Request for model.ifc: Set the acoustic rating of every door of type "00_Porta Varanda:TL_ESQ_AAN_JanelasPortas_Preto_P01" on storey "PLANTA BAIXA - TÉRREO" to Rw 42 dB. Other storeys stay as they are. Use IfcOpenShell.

First a look at what the model holds.

```python
import ifcopenshell
import ifcopenshell.util.element

model = ifcopenshell.open("model.ifc")
print(model.schema)
storey = next(s for s in model.by_type("IfcBuildingStorey") if s.Name == "PLANTA BAIXA - TÉRREO")
doors = [e for e in ifcopenshell.util.element.get_decomposition(storey) if e.is_a("IfcDoor")]
seen = {}
for e in doors:
    element_type = ifcopenshell.util.element.get_type(e)
    key = (element_type.Name if element_type != e and element_type else None, ifcopenshell.util.element.get_pset(e, "Pset_DoorCommon", "AcousticRating"))
    seen[key] = seen.get(key, 0) + 1
for (name, value), count in sorted(seen.items(), key=str):
    print(count, "x", name, "|", value)
```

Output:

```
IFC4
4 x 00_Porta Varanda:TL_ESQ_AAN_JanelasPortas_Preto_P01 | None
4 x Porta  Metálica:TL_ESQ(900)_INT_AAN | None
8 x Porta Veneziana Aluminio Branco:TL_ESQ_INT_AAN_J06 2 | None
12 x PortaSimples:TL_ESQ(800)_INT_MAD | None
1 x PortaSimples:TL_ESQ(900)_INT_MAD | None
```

```python
import ifcopenshell
import ifcopenshell.api.pset
import ifcopenshell.util.element

model = ifcopenshell.open("model.ifc")

storey = next(s for s in model.by_type("IfcBuildingStorey") if s.Name == "PLANTA BAIXA - TÉRREO")
doors = [e for e in ifcopenshell.util.element.get_decomposition(storey) if e.is_a("IfcDoor")]

count = 0
for e in doors:
    element_type = ifcopenshell.util.element.get_type(e)
    if element_type in (None, e) or element_type.Name != "00_Porta Varanda:TL_ESQ_AAN_JanelasPortas_Preto_P01":
        continue
    # add_pset returns the element's existing set when there is one.
    pset = ifcopenshell.api.pset.add_pset(model, product=e, name="Pset_DoorCommon")
    ifcopenshell.api.pset.edit_pset(model, pset=pset, properties={"AcousticRating": "Rw 42 dB"})
    count += 1

print(count, "doors updated")

model.write("model_edited.ifc")
```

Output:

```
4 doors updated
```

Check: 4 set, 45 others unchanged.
